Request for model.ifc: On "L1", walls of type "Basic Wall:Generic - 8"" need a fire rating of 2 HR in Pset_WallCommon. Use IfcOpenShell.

First a look at what the model holds.

```python
import ifcopenshell
import ifcopenshell.util.element

model = ifcopenshell.open("model.ifc")
print(model.schema)
storey = next(s for s in model.by_type("IfcBuildingStorey") if s.Name == "L1")
walls = [e for e in ifcopenshell.util.element.get_decomposition(storey) if e.is_a("IfcWall")]
seen = {}
for e in walls:
    element_type = ifcopenshell.util.element.get_type(e)
    key = (element_type.Name if element_type != e and element_type else None, ifcopenshell.util.element.get_pset(e, "Pset_WallCommon", "FireRating"))
    seen[key] = seen.get(key, 0) + 1
for (name, value), count in sorted(seen.items(), key=str):
    print(count, "x", name, "|", value)
```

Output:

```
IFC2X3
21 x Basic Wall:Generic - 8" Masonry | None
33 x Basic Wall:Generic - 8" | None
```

```python
import ifcopenshell
import ifcopenshell.api.pset
import ifcopenshell.util.element

model = ifcopenshell.open("model.ifc")

storey = next(s for s in model.by_type("IfcBuildingStorey") if s.Name == "L1")
walls = [e for e in ifcopenshell.util.element.get_decomposition(storey) if e.is_a("IfcWall")]

count = 0
for e in walls:
    element_type = ifcopenshell.util.element.get_type(e)
    if element_type in (None, e) or element_type.Name != 'Basic Wall:Generic - 8"':
        continue
    # add_pset returns the element's existing set when there is one.
    pset = ifcopenshell.api.pset.add_pset(model, product=e, name="Pset_WallCommon")
    ifcopenshell.api.pset.edit_pset(model, pset=pset, properties={"FireRating": "2 HR"})
    count += 1

print(count, "walls updated")

model.write("model_v2.ifc")
```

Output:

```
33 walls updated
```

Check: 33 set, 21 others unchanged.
